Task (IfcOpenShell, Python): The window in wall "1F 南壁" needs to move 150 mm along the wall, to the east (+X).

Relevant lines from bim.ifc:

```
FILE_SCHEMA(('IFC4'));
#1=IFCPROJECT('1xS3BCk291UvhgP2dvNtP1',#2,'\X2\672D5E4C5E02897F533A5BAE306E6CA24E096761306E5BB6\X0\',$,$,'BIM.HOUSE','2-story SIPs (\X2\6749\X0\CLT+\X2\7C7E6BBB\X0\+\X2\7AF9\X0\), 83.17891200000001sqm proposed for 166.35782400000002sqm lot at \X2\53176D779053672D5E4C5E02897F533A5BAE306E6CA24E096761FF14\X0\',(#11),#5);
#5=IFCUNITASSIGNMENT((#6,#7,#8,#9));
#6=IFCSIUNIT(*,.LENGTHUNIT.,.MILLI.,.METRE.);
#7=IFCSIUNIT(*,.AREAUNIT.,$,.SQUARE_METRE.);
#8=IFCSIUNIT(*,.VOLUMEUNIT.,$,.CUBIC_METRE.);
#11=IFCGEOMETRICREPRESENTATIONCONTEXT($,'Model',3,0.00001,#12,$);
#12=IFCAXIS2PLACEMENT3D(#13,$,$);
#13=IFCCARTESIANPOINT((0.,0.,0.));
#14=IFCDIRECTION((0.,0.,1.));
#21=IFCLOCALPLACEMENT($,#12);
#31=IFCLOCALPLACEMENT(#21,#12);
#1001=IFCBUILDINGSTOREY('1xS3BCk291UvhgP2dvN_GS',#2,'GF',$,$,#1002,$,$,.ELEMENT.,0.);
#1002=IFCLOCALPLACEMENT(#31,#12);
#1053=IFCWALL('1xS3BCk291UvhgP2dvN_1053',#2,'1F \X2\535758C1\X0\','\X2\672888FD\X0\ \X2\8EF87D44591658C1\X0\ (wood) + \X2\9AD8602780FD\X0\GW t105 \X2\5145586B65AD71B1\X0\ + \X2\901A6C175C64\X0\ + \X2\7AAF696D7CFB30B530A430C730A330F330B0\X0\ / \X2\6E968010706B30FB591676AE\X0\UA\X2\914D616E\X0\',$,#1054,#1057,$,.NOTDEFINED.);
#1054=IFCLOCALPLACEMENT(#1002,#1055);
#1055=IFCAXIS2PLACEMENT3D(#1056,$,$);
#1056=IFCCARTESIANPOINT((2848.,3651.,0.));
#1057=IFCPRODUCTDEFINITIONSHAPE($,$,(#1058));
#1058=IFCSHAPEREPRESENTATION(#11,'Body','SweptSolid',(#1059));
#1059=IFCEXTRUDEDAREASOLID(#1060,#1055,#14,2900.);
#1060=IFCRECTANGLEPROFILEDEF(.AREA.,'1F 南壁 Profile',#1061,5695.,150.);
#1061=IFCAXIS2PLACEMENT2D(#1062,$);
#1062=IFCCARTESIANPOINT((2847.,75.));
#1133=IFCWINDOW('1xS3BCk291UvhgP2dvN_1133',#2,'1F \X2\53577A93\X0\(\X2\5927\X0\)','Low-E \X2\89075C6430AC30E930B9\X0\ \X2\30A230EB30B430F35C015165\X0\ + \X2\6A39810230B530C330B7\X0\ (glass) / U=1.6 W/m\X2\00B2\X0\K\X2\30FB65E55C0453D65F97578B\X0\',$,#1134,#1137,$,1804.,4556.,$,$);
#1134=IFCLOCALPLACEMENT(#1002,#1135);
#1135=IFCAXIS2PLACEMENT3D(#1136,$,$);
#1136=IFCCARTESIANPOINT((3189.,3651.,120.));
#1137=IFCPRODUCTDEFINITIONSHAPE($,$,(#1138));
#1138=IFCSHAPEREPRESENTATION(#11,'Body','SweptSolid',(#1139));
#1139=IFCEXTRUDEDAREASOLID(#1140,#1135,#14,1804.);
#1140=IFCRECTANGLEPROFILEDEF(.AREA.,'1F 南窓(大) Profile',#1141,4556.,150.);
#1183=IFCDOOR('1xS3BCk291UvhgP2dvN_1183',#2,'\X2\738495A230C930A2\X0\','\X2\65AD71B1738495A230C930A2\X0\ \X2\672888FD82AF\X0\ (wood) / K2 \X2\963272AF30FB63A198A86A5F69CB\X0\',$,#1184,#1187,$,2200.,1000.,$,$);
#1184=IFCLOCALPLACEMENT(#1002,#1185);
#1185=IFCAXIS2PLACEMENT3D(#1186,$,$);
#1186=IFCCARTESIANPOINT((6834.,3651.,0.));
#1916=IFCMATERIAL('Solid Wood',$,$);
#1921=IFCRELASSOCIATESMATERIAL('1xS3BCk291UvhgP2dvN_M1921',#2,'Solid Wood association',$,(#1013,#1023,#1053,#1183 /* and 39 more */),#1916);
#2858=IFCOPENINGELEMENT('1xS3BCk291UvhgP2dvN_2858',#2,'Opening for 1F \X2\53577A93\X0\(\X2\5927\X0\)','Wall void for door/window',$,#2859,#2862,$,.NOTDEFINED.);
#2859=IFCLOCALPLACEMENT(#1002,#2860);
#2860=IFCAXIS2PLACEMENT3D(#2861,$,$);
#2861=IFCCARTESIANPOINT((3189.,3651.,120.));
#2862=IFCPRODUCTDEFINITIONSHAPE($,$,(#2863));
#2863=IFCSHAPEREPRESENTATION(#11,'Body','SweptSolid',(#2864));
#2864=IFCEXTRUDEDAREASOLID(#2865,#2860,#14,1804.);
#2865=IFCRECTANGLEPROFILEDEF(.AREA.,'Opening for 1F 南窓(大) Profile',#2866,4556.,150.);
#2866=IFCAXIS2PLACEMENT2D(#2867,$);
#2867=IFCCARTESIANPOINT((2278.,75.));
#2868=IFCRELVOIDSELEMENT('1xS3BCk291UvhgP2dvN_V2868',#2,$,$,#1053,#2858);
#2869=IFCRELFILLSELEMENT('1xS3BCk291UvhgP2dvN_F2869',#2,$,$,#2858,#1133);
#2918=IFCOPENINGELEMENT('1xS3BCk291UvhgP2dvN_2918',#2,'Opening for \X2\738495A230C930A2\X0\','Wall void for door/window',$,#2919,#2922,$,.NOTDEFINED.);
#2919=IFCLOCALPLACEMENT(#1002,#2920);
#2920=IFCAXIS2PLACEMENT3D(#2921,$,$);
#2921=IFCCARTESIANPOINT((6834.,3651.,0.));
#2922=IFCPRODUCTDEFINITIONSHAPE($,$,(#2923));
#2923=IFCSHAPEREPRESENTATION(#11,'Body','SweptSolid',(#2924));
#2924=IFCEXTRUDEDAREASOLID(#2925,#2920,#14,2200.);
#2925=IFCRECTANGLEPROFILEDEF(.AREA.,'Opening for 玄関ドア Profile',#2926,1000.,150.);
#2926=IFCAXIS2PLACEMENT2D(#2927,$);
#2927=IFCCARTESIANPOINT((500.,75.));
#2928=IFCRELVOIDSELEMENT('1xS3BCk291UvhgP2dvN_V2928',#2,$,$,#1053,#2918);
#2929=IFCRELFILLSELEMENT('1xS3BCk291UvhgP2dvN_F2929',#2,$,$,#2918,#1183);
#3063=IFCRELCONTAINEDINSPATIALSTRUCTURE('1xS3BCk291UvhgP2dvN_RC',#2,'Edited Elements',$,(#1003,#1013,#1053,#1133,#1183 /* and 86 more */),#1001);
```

```python
import ifcopenshell
import ifcopenshell.api.geometry
import ifcopenshell.util.placement
import ifcopenshell.util.unit

model = ifcopenshell.open("bim.ifc")
unit_scale = ifcopenshell.util.unit.calculate_unit_scale(model)

window = model.by_guid("1xS3BCk291UvhgP2dvN_1133")
opening = window.FillsVoids[0].RelatingOpeningElement
wall = opening.VoidsElements[0].RelatingBuildingElement

wall_matrix = ifcopenshell.util.placement.get_local_placement(wall.ObjectPlacement)
shift = wall_matrix[:3, 0] * 0.15 / unit_scale
before = ifcopenshell.util.placement.get_local_placement(window.ObjectPlacement)[:3, 3].copy()

# The window is not placed relative to its opening, so move both.
for product in (opening, window):
    matrix = ifcopenshell.util.placement.get_local_placement(product.ObjectPlacement)
    matrix[:3, 3] += shift
    ifcopenshell.api.geometry.edit_object_placement(model, product=product, matrix=matrix, is_si=False)

after = ifcopenshell.util.placement.get_local_placement(window.ObjectPlacement)[:3, 3]
print("window moved by", (after - before).round(3) + 0.0)

model.write("bim_v2.ifc")
```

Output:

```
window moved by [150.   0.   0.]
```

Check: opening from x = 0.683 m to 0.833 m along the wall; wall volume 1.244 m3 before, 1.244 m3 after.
